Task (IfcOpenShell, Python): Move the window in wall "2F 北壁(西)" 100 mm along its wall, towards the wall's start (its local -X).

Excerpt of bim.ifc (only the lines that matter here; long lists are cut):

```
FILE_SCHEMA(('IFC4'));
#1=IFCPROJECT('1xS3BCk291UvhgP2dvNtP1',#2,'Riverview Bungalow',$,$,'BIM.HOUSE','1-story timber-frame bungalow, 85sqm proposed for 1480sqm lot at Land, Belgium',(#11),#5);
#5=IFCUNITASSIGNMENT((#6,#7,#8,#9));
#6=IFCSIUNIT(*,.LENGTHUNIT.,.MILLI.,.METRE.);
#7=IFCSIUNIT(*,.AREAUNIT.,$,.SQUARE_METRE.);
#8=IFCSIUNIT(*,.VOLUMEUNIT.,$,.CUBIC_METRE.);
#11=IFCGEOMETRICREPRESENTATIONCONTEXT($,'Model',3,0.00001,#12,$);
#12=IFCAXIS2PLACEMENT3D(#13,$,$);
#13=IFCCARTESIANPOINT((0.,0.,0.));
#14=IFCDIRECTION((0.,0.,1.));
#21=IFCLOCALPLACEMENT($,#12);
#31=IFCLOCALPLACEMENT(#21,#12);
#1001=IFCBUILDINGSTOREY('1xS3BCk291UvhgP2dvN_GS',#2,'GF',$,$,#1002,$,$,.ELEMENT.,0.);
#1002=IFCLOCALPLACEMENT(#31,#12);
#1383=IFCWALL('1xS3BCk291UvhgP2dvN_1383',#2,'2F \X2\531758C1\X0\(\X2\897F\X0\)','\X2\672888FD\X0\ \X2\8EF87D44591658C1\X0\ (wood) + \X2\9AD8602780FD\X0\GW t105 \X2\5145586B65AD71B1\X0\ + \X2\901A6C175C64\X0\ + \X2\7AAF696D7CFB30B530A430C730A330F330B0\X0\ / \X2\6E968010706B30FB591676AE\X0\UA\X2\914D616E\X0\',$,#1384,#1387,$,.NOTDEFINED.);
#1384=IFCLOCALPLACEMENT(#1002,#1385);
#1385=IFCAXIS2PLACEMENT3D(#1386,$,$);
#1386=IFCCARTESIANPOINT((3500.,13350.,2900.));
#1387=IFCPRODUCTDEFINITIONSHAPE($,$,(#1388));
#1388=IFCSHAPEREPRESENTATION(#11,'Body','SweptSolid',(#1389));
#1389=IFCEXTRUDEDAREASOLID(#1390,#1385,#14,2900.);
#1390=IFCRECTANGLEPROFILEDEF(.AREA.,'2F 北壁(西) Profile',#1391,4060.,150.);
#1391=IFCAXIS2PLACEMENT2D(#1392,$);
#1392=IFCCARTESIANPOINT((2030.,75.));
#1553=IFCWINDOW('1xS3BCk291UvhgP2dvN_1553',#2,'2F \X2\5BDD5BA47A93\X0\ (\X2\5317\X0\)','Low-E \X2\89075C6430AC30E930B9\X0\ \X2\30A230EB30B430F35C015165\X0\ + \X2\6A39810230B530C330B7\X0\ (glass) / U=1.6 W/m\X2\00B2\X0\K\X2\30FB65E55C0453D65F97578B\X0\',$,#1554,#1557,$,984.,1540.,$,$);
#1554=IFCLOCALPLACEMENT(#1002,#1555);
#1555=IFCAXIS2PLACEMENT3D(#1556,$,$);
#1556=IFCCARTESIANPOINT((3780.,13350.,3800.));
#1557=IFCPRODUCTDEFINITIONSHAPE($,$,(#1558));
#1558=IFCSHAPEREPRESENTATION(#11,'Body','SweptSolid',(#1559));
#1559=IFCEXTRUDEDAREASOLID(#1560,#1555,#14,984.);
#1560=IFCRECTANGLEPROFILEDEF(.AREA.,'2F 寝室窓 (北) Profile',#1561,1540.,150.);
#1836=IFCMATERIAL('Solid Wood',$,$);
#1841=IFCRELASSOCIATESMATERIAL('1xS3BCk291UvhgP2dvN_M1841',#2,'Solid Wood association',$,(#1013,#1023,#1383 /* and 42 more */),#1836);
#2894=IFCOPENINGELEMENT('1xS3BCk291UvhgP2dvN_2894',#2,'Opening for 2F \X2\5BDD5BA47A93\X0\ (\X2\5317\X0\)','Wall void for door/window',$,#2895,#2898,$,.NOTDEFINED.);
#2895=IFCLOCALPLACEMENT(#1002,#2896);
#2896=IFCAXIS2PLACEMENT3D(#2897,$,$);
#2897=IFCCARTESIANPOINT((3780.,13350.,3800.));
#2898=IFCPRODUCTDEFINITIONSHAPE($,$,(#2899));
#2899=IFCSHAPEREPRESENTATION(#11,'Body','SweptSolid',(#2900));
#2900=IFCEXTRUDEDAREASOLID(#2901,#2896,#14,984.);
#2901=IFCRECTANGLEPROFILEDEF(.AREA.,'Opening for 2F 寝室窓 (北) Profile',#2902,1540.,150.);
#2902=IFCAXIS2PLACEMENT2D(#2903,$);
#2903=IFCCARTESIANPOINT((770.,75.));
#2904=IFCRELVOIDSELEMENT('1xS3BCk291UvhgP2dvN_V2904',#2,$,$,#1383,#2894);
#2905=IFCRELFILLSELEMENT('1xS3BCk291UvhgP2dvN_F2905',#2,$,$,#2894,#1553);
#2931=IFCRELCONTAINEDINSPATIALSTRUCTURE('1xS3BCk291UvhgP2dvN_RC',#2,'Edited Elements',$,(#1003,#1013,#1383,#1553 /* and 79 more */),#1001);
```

```python
import ifcopenshell
import ifcopenshell.api.geometry
import ifcopenshell.util.placement
import ifcopenshell.util.unit

model = ifcopenshell.open("bim.ifc")
unit_scale = ifcopenshell.util.unit.calculate_unit_scale(model)

window = model.by_guid("1xS3BCk291UvhgP2dvN_1553")
opening = window.FillsVoids[0].RelatingOpeningElement
wall = opening.VoidsElements[0].RelatingBuildingElement

wall_matrix = ifcopenshell.util.placement.get_local_placement(wall.ObjectPlacement)
shift = wall_matrix[:3, 0] * -0.1 / unit_scale
before = ifcopenshell.util.placement.get_local_placement(window.ObjectPlacement)[:3, 3].copy()

# The window is not placed relative to its opening, so move both.
for product in (opening, window):
    matrix = ifcopenshell.util.placement.get_local_placement(product.ObjectPlacement)
    matrix[:3, 3] += shift
    ifcopenshell.api.geometry.edit_object_placement(model, product=product, matrix=matrix, is_si=False)

after = ifcopenshell.util.placement.get_local_placement(window.ObjectPlacement)[:3, 3]
print("window moved by", (after - before).round(3) + 0.0)

model.write("bim_v2.ifc")
```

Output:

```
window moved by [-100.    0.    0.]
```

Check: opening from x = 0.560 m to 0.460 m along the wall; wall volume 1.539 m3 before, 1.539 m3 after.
